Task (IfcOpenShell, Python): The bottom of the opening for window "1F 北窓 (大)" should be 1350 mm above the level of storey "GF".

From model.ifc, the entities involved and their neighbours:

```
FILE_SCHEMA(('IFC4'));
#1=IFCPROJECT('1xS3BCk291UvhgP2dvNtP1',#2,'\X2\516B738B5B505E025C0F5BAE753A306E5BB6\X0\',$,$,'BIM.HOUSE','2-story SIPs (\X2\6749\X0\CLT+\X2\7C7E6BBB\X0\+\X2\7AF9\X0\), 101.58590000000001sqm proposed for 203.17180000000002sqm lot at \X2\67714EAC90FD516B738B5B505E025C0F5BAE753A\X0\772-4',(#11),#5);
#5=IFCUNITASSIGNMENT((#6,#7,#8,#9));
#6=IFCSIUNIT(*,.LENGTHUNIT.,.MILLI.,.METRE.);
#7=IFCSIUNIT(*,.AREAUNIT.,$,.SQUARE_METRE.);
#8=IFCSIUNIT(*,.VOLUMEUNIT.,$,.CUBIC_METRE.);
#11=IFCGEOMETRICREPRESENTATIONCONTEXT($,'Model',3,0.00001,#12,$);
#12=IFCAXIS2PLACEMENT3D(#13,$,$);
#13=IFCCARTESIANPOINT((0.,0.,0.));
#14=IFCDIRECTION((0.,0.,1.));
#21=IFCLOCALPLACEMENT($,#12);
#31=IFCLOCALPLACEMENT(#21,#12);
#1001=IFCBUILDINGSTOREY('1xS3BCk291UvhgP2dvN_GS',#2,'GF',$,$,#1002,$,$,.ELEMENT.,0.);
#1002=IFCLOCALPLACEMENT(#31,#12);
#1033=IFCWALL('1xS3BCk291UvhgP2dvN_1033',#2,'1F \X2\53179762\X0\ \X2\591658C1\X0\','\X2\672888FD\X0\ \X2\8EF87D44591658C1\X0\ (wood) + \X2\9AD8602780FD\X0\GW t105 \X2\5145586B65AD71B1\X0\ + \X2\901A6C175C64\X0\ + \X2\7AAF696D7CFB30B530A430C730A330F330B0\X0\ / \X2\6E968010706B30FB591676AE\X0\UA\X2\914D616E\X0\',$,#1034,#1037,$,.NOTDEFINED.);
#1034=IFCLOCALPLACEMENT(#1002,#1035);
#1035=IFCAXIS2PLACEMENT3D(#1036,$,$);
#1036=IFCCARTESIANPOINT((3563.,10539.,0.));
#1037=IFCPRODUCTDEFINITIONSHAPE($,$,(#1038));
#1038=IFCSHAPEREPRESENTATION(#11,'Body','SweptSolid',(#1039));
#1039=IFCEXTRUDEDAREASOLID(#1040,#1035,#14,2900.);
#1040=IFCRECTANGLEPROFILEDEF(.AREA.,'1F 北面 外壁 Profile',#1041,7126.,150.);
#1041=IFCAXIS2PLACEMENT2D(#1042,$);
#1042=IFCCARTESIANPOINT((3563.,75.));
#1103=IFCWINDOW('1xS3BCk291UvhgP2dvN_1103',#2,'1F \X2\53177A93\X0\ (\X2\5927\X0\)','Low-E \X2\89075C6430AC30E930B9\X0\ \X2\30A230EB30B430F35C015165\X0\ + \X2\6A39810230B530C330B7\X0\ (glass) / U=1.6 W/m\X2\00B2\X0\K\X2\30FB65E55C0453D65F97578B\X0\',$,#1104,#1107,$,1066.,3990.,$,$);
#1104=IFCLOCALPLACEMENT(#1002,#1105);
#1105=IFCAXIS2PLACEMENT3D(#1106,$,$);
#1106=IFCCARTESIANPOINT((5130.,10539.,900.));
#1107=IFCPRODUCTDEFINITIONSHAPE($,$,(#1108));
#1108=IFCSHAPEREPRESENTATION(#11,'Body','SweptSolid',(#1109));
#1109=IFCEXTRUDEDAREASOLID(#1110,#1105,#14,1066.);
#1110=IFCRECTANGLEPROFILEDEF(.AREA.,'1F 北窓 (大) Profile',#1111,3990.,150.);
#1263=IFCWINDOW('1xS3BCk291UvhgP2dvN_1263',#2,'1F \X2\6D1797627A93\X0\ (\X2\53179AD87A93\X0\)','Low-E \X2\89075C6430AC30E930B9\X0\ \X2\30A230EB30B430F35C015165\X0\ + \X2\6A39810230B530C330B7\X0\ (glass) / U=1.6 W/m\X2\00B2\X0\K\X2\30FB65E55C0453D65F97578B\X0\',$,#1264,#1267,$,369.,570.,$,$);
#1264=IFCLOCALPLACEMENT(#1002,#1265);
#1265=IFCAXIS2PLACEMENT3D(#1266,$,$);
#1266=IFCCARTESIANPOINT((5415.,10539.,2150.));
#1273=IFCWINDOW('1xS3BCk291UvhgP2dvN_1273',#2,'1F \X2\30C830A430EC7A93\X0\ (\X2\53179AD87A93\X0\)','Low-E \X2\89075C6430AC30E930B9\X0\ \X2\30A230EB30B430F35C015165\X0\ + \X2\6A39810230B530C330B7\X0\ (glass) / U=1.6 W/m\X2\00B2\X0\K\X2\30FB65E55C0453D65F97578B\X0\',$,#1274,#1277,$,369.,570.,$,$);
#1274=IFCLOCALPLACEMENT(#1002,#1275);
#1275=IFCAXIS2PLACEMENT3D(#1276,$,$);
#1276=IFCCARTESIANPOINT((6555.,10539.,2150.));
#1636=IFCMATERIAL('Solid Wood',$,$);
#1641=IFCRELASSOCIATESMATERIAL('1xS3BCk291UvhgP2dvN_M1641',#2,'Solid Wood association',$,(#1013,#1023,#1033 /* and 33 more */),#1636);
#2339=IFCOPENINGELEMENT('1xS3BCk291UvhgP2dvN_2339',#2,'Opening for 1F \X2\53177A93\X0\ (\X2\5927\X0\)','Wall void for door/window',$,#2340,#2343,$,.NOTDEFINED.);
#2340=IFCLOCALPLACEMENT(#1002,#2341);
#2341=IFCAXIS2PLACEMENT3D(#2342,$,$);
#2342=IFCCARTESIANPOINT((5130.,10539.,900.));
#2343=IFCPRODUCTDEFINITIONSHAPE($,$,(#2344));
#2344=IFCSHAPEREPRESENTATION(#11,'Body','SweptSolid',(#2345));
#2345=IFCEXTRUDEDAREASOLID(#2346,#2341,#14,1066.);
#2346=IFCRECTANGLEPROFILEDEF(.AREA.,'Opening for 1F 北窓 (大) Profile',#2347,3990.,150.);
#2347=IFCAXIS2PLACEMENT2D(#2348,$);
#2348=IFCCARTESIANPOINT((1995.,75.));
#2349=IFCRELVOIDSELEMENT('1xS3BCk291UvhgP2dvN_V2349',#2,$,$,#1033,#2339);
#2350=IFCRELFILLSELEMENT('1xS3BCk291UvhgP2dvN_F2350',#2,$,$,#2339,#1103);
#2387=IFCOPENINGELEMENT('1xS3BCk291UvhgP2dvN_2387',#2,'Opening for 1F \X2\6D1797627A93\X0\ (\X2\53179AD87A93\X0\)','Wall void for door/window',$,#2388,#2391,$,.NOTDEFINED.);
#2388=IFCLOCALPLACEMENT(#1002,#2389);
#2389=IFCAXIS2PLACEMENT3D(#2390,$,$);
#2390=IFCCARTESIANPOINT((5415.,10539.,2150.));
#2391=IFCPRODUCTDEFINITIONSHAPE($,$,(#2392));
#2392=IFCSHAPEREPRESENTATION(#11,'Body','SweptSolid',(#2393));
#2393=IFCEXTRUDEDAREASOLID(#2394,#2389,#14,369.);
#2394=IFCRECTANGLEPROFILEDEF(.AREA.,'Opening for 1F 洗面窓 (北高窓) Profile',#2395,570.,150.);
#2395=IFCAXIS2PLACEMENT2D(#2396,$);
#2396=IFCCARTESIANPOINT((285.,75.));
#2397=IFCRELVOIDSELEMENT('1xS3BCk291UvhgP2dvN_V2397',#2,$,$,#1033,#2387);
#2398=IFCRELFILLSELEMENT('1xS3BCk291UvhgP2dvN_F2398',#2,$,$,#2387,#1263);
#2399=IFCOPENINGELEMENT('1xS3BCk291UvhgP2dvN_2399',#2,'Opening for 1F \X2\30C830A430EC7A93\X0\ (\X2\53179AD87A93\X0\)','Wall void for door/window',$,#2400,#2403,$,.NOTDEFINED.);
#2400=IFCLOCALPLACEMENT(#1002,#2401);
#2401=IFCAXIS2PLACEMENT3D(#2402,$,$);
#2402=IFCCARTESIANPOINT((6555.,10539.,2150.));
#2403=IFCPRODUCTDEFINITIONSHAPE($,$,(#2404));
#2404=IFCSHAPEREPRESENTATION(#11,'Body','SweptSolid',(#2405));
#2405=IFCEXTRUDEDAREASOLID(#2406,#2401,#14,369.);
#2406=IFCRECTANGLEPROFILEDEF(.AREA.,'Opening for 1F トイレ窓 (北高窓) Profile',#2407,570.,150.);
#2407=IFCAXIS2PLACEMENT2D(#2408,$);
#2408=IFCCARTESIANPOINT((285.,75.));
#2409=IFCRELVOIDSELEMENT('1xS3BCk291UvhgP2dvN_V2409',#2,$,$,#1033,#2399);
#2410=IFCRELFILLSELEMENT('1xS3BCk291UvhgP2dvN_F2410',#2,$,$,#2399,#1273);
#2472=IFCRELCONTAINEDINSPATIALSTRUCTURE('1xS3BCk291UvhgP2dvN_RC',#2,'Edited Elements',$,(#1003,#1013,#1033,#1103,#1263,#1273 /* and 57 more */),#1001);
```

```python
import numpy as np
import ifcopenshell
import ifcopenshell.api.geometry
import ifcopenshell.geom
import ifcopenshell.util.element
import ifcopenshell.util.placement
import ifcopenshell.util.shape
import ifcopenshell.util.unit

model = ifcopenshell.open("model.ifc")
unit_scale = ifcopenshell.util.unit.calculate_unit_scale(model)

window = model.by_guid("1xS3BCk291UvhgP2dvN_1103")
opening = window.FillsVoids[0].RelatingOpeningElement
storey = ifcopenshell.util.element.get_container(window, ifc_class="IfcBuildingStorey")
level = ifcopenshell.util.placement.get_local_placement(storey.ObjectPlacement)[2, 3]

# The opening's origin need not be at the sill, so measure its lowest point.
shape = ifcopenshell.geom.create_shape(ifcopenshell.geom.settings(), opening)
bottom = ifcopenshell.util.shape.get_shape_bottom_elevation(shape, shape.geometry) / unit_scale
dz = level + 1.35 / unit_scale - bottom

shift = np.array([0.0, 0.0, dz])
# The window is not placed relative to its opening, so move both.
for product in (opening, window):
    matrix = ifcopenshell.util.placement.get_local_placement(product.ObjectPlacement)
    matrix[:3, 3] += shift
    ifcopenshell.api.geometry.edit_object_placement(model, product=product, matrix=matrix, is_si=False)

print(f"moved by {dz * unit_scale:+.3f} m")

model.write("model_edited.ifc")
```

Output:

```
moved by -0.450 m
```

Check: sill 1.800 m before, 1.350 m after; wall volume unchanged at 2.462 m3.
